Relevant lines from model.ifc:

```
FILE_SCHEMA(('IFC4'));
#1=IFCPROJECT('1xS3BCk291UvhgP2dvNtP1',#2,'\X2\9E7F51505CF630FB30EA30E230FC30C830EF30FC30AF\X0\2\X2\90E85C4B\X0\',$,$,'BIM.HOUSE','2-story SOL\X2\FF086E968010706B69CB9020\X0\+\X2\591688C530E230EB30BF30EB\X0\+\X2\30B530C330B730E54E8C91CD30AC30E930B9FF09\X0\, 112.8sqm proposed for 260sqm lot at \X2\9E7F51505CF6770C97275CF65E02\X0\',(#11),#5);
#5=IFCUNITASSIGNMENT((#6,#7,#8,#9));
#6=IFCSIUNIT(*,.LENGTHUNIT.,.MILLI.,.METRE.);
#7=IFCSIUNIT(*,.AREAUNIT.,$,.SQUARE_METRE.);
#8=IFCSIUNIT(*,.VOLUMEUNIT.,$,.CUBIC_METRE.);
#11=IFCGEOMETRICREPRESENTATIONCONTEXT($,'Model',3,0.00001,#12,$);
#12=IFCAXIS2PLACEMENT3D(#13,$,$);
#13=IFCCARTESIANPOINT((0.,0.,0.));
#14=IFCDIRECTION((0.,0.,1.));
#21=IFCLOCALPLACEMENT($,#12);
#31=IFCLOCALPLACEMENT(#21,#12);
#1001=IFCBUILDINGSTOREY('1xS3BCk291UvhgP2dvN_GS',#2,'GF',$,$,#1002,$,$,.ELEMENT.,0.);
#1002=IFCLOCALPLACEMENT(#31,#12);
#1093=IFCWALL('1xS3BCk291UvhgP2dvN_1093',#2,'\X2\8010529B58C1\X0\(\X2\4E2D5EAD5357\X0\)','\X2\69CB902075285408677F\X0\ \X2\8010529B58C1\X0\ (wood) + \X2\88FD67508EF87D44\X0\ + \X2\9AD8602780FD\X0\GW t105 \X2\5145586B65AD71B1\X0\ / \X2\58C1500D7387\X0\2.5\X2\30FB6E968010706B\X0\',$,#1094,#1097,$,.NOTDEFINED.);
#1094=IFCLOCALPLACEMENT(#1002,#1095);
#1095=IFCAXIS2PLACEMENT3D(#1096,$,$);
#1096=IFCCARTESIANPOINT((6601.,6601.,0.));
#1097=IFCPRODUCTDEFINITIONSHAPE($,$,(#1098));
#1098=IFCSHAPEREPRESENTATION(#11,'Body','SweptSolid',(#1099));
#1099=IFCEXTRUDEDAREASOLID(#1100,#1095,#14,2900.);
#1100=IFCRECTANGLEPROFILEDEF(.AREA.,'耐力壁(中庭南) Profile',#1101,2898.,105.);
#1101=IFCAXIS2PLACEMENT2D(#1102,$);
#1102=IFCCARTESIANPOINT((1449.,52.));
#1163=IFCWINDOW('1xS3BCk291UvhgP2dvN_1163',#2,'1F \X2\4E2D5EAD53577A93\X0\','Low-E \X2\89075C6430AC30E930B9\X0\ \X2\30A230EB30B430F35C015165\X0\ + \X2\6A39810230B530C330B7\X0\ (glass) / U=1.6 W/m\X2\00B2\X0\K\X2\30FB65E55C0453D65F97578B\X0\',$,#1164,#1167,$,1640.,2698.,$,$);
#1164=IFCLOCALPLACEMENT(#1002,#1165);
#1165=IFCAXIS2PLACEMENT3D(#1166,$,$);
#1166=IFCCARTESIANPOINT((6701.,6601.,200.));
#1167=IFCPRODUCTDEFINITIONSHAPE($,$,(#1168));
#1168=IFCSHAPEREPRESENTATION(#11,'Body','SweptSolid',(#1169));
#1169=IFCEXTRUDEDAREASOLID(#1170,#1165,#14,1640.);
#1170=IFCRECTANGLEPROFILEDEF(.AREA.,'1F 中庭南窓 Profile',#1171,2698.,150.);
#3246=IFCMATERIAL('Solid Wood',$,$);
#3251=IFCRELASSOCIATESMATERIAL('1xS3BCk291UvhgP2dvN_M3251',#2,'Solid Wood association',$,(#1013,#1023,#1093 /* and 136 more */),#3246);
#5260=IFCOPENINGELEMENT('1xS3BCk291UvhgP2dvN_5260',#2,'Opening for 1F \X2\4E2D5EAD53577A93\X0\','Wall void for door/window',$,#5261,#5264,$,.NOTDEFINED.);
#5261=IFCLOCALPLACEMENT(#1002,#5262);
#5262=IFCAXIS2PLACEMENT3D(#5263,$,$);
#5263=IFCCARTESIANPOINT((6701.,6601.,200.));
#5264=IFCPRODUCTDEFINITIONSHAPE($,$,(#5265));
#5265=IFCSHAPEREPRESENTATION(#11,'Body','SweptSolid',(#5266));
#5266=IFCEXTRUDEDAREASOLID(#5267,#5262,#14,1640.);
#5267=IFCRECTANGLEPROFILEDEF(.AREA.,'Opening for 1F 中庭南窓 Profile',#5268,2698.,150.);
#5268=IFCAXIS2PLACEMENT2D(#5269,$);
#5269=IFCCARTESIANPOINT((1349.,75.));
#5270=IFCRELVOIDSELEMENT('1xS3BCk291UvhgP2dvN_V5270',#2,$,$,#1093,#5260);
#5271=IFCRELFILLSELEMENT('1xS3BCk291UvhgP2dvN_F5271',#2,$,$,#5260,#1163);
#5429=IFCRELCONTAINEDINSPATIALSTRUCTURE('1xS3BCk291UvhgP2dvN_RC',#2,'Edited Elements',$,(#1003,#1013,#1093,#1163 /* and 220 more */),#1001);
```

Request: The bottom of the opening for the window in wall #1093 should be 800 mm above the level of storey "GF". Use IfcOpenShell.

```python
import numpy as np
import ifcopenshell
import ifcopenshell.api.geometry
import ifcopenshell.geom
import ifcopenshell.util.element
import ifcopenshell.util.placement
import ifcopenshell.util.shape
import ifcopenshell.util.unit

model = ifcopenshell.open("model.ifc")
unit_scale = ifcopenshell.util.unit.calculate_unit_scale(model)

window = model.by_guid("1xS3BCk291UvhgP2dvN_1163")
opening = window.FillsVoids[0].RelatingOpeningElement
storey = ifcopenshell.util.element.get_container(window, ifc_class="IfcBuildingStorey")
level = ifcopenshell.util.placement.get_local_placement(storey.ObjectPlacement)[2, 3]

# The opening's origin need not be at the sill, so measure its lowest point.
shape = ifcopenshell.geom.create_shape(ifcopenshell.geom.settings(), opening)
bottom = ifcopenshell.util.shape.get_shape_bottom_elevation(shape, shape.geometry) / unit_scale
dz = level + 800.0 - bottom

shift = np.array([0.0, 0.0, dz])
# The window is not placed relative to its opening, so move both.
for product in (opening, window):
    matrix = ifcopenshell.util.placement.get_local_placement(product.ObjectPlacement)
    matrix[:3, 3] += shift
    ifcopenshell.api.geometry.edit_object_placement(model, product=product, matrix=matrix, is_si=False)

print(f"moved by {dz * unit_scale:+.3f} m")

model.write("model_updated.ifc")
```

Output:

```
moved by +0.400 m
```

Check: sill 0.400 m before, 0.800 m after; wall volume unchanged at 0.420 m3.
